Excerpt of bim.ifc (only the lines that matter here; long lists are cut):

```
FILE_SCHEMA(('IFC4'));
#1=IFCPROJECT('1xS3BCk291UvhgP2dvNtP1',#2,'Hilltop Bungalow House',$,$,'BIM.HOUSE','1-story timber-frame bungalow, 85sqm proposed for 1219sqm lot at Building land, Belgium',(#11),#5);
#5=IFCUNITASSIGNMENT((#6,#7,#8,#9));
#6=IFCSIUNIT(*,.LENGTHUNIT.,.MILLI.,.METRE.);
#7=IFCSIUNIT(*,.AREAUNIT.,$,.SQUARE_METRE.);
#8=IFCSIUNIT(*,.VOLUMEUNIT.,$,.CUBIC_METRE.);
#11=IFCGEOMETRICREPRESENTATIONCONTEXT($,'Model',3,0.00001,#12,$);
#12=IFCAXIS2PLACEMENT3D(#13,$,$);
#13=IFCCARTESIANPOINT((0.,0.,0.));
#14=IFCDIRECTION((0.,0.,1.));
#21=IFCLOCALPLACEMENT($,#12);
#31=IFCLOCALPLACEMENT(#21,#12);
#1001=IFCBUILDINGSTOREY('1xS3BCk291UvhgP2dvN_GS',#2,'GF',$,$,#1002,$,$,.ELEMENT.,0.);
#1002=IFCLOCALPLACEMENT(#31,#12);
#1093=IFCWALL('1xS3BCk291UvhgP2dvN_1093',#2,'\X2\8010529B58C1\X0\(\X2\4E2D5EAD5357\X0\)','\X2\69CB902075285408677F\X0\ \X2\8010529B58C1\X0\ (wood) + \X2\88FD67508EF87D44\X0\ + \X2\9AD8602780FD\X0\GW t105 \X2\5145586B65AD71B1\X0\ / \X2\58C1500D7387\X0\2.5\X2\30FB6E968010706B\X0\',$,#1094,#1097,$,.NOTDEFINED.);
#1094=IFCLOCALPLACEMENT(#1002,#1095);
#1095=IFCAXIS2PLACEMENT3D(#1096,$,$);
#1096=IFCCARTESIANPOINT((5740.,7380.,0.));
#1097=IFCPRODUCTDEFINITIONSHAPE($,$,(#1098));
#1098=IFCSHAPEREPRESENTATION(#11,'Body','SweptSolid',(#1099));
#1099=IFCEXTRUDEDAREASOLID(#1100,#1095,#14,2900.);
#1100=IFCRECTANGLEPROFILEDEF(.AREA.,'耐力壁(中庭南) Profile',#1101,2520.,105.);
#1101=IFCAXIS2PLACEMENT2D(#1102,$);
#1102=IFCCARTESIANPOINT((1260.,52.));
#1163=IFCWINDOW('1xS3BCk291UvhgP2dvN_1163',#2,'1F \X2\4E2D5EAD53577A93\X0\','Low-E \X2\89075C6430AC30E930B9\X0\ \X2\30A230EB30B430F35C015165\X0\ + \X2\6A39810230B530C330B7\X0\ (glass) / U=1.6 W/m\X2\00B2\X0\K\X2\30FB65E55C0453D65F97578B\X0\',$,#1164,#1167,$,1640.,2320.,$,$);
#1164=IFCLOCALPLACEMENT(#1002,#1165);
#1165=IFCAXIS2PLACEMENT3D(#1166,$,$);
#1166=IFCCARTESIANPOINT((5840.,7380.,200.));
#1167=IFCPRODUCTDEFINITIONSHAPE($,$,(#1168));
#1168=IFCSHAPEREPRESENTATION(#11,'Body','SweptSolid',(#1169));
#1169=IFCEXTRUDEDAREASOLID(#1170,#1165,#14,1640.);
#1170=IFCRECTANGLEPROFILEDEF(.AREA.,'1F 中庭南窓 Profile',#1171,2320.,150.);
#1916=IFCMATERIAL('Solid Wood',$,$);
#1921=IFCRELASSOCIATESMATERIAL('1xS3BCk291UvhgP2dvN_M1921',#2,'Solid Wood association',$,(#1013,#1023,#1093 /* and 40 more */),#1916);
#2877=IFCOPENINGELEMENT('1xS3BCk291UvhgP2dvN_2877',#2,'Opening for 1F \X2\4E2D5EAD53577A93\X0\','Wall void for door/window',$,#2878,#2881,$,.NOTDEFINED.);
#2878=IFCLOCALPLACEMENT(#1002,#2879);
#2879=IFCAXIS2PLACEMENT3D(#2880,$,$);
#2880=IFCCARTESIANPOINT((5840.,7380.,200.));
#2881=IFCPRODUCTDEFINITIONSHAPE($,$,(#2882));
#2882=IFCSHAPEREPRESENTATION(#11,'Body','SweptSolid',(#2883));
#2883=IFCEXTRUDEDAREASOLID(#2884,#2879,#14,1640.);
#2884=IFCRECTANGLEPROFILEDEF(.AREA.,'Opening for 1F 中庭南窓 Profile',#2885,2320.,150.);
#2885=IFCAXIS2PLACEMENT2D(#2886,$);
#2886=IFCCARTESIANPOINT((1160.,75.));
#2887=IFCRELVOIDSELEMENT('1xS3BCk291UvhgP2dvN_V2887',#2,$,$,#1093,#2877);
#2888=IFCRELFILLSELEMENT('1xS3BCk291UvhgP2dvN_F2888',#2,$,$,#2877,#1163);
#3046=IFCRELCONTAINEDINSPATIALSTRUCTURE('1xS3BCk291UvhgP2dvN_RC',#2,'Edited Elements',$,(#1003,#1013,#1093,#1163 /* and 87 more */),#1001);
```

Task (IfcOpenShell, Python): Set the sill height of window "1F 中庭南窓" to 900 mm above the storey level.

```python
import numpy as np
import ifcopenshell
import ifcopenshell.api.geometry
import ifcopenshell.geom
import ifcopenshell.util.element
import ifcopenshell.util.placement
import ifcopenshell.util.shape
import ifcopenshell.util.unit

model = ifcopenshell.open("bim.ifc")
unit_scale = ifcopenshell.util.unit.calculate_unit_scale(model)

window = model.by_guid("1xS3BCk291UvhgP2dvN_1163")
opening = window.FillsVoids[0].RelatingOpeningElement
storey = ifcopenshell.util.element.get_container(window, ifc_class="IfcBuildingStorey")
level = ifcopenshell.util.placement.get_local_placement(storey.ObjectPlacement)[2, 3]

# The opening's origin need not be at the sill, so measure its lowest point.
shape = ifcopenshell.geom.create_shape(ifcopenshell.geom.settings(), opening)
bottom = ifcopenshell.util.shape.get_shape_bottom_elevation(shape, shape.geometry) / unit_scale
dz = level + 900.0 - bottom

shift = np.array([0.0, 0.0, dz])
# The window is not placed relative to its opening, so move both.
for product in (opening, window):
    matrix = ifcopenshell.util.placement.get_local_placement(product.ObjectPlacement)
    matrix[:3, 3] += shift
    ifcopenshell.api.geometry.edit_object_placement(model, product=product, matrix=matrix, is_si=False)

print(f"moved by {dz * unit_scale:+.3f} m")

model.write("bim-out.ifc")
```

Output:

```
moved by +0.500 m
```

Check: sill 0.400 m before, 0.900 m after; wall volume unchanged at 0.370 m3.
